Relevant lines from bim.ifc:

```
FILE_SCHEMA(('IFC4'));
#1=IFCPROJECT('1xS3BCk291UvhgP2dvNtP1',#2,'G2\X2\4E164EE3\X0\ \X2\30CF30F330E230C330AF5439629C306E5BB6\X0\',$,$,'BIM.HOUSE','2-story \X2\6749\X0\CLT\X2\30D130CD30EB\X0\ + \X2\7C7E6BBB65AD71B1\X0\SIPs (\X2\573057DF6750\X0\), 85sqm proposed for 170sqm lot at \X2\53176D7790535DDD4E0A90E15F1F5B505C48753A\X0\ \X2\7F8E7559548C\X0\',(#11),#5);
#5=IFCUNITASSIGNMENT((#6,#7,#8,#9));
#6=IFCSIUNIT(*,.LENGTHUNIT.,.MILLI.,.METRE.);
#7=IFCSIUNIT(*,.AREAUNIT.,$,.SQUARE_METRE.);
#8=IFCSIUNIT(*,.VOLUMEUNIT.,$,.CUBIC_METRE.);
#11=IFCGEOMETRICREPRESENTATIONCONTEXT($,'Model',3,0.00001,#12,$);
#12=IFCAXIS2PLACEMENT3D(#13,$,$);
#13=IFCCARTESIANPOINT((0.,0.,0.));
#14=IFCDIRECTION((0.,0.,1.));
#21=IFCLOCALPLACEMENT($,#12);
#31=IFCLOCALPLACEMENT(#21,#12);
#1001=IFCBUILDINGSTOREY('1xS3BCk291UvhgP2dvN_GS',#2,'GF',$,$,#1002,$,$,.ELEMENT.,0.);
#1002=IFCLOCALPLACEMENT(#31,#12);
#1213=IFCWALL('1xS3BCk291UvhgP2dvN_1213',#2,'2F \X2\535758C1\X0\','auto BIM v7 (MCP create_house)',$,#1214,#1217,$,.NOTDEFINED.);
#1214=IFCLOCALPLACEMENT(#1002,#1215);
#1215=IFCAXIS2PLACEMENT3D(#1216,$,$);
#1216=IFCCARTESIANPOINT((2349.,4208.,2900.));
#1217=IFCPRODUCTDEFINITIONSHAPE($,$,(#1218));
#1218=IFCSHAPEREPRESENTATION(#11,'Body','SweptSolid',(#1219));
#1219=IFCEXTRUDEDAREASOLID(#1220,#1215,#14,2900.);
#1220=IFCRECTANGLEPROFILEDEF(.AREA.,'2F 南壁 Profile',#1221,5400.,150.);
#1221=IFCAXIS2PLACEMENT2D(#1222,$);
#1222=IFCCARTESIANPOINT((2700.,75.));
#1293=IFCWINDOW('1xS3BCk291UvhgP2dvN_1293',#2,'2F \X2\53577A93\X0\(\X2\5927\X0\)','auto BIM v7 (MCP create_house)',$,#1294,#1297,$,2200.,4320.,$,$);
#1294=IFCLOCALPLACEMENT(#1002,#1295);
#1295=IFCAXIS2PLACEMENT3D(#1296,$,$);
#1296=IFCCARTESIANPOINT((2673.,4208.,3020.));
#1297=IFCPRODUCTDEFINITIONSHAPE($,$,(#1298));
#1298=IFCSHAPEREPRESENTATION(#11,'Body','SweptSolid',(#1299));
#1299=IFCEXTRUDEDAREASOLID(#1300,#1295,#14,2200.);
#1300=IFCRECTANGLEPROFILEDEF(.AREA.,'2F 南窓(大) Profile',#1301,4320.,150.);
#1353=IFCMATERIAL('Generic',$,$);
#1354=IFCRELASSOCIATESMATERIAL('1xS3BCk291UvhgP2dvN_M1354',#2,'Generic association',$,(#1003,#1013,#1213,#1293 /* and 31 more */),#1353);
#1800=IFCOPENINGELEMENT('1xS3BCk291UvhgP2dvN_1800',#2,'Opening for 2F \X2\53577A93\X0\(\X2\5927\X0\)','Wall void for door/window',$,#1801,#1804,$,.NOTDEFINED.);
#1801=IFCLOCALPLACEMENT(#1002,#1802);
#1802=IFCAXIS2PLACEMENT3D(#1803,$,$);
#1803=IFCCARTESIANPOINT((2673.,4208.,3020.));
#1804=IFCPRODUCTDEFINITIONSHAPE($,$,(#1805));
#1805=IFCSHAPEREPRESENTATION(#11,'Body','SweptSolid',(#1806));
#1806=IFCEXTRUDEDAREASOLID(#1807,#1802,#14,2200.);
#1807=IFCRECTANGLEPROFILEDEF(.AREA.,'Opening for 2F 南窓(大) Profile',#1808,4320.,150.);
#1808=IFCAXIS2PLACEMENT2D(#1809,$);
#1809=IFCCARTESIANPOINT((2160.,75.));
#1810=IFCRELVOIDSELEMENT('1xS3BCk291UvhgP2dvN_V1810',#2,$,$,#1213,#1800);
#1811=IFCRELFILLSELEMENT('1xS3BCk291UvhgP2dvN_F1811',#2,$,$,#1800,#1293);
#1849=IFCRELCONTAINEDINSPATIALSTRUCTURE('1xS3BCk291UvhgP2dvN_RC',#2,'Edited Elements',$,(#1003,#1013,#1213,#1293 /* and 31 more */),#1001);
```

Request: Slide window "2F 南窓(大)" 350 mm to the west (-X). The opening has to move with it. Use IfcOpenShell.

```python
import ifcopenshell
import ifcopenshell.api.geometry
import ifcopenshell.util.placement
import ifcopenshell.util.unit

model = ifcopenshell.open("bim.ifc")
unit_scale = ifcopenshell.util.unit.calculate_unit_scale(model)

window = model.by_guid("1xS3BCk291UvhgP2dvN_1293")
opening = window.FillsVoids[0].RelatingOpeningElement
wall = opening.VoidsElements[0].RelatingBuildingElement

wall_matrix = ifcopenshell.util.placement.get_local_placement(wall.ObjectPlacement)
shift = wall_matrix[:3, 0] * -0.35 / unit_scale
before = ifcopenshell.util.placement.get_local_placement(window.ObjectPlacement)[:3, 3].copy()

# The window is not placed relative to its opening, so move both.
for product in (opening, window):
    matrix = ifcopenshell.util.placement.get_local_placement(product.ObjectPlacement)
    matrix[:3, 3] += shift
    ifcopenshell.api.geometry.edit_object_placement(model, product=product, matrix=matrix, is_si=False)

after = ifcopenshell.util.placement.get_local_placement(window.ObjectPlacement)[:3, 3]
print("window moved by", (after - before).round(3) + 0.0)

model.write("bim-out.ifc")
```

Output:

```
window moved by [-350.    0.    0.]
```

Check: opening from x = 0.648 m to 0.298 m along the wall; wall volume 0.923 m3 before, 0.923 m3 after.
